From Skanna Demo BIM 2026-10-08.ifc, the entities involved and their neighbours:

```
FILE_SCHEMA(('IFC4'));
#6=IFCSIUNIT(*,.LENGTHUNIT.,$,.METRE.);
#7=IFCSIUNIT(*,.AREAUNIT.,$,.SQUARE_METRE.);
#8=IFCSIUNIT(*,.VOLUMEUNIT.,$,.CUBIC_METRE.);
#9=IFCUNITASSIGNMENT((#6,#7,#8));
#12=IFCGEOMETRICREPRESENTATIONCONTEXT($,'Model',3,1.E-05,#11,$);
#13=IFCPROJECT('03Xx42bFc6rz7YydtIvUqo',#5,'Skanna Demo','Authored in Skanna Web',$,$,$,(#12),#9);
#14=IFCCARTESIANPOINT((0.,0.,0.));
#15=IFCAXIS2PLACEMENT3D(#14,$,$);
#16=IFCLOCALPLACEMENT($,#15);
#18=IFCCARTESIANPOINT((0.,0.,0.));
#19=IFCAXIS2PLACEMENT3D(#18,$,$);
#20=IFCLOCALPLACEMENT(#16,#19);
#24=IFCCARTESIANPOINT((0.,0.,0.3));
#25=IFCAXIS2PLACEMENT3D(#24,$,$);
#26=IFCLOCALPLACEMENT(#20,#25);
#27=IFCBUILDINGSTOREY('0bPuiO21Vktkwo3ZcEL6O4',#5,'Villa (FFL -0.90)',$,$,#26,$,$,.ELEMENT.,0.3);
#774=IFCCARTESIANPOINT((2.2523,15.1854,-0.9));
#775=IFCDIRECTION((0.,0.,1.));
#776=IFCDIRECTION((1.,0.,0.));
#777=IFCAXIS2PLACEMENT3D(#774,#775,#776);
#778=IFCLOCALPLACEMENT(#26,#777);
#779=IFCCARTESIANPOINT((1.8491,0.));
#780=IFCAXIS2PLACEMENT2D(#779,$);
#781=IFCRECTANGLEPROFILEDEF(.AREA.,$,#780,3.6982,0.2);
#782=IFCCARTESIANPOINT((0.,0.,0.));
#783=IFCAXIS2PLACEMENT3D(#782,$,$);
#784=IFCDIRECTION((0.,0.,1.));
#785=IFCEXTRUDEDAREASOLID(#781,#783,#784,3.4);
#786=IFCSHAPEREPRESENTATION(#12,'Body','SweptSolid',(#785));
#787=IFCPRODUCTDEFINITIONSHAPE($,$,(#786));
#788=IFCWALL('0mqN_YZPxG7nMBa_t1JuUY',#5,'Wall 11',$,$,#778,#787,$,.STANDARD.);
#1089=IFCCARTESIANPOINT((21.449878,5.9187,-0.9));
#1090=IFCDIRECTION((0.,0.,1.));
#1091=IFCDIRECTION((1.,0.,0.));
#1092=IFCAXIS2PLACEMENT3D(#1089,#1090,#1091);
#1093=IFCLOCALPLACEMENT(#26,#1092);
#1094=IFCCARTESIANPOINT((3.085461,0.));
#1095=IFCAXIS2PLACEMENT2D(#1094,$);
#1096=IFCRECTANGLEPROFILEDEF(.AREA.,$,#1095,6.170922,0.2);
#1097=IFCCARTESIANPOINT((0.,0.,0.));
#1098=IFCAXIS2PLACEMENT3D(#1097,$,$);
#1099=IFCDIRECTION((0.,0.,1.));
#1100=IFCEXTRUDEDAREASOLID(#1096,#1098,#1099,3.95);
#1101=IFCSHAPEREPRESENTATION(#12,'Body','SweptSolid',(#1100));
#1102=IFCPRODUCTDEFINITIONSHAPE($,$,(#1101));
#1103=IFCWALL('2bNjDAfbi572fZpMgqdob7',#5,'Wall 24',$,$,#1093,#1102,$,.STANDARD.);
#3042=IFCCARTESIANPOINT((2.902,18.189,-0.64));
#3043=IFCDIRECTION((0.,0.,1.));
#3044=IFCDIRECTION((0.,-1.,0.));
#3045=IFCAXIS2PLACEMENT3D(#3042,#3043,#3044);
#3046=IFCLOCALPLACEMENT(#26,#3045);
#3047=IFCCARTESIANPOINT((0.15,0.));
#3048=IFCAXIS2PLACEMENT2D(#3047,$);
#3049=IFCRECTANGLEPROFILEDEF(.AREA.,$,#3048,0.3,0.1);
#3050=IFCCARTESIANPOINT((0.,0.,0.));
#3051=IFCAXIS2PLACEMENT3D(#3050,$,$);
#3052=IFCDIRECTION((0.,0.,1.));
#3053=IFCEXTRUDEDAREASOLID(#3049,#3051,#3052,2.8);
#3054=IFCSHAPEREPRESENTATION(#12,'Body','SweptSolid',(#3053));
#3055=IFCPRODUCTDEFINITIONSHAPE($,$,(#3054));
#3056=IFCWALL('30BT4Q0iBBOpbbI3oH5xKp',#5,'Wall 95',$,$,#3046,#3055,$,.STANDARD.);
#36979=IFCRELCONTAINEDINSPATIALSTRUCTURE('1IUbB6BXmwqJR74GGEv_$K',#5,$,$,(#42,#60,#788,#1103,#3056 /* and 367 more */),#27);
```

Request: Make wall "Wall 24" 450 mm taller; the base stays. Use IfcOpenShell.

```python
import ifcopenshell
import ifcopenshell.geom
import ifcopenshell.util.shape
import ifcopenshell.util.unit

model = ifcopenshell.open("Skanna Demo BIM 2026-10-08.ifc")
unit_scale = ifcopenshell.util.unit.calculate_unit_scale(model)
settings = ifcopenshell.geom.settings()


def volume(element):
    """Net volume in cubic metres, openings subtracted."""
    shape = ifcopenshell.geom.create_shape(settings, element)
    return ifcopenshell.util.shape.get_volume(shape.geometry)


wall = model.by_guid("2bNjDAfbi572fZpMgqdob7")
before = volume(wall)

body = next(r for r in wall.Representation.Representations if r.RepresentationIdentifier == "Body")
solid = body.Items[0]
old_height = solid.Depth
solid.Depth += 0.45 / unit_scale
after = volume(wall)

print(f"height {old_height:g} -> {solid.Depth:g}, volume {before:.3f} -> {after:.3f} m3")

model.write("Skanna Demo BIM 2026-10-08_rev.ifc")
```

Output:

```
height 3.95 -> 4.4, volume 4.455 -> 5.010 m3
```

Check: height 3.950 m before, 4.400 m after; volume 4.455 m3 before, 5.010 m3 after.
